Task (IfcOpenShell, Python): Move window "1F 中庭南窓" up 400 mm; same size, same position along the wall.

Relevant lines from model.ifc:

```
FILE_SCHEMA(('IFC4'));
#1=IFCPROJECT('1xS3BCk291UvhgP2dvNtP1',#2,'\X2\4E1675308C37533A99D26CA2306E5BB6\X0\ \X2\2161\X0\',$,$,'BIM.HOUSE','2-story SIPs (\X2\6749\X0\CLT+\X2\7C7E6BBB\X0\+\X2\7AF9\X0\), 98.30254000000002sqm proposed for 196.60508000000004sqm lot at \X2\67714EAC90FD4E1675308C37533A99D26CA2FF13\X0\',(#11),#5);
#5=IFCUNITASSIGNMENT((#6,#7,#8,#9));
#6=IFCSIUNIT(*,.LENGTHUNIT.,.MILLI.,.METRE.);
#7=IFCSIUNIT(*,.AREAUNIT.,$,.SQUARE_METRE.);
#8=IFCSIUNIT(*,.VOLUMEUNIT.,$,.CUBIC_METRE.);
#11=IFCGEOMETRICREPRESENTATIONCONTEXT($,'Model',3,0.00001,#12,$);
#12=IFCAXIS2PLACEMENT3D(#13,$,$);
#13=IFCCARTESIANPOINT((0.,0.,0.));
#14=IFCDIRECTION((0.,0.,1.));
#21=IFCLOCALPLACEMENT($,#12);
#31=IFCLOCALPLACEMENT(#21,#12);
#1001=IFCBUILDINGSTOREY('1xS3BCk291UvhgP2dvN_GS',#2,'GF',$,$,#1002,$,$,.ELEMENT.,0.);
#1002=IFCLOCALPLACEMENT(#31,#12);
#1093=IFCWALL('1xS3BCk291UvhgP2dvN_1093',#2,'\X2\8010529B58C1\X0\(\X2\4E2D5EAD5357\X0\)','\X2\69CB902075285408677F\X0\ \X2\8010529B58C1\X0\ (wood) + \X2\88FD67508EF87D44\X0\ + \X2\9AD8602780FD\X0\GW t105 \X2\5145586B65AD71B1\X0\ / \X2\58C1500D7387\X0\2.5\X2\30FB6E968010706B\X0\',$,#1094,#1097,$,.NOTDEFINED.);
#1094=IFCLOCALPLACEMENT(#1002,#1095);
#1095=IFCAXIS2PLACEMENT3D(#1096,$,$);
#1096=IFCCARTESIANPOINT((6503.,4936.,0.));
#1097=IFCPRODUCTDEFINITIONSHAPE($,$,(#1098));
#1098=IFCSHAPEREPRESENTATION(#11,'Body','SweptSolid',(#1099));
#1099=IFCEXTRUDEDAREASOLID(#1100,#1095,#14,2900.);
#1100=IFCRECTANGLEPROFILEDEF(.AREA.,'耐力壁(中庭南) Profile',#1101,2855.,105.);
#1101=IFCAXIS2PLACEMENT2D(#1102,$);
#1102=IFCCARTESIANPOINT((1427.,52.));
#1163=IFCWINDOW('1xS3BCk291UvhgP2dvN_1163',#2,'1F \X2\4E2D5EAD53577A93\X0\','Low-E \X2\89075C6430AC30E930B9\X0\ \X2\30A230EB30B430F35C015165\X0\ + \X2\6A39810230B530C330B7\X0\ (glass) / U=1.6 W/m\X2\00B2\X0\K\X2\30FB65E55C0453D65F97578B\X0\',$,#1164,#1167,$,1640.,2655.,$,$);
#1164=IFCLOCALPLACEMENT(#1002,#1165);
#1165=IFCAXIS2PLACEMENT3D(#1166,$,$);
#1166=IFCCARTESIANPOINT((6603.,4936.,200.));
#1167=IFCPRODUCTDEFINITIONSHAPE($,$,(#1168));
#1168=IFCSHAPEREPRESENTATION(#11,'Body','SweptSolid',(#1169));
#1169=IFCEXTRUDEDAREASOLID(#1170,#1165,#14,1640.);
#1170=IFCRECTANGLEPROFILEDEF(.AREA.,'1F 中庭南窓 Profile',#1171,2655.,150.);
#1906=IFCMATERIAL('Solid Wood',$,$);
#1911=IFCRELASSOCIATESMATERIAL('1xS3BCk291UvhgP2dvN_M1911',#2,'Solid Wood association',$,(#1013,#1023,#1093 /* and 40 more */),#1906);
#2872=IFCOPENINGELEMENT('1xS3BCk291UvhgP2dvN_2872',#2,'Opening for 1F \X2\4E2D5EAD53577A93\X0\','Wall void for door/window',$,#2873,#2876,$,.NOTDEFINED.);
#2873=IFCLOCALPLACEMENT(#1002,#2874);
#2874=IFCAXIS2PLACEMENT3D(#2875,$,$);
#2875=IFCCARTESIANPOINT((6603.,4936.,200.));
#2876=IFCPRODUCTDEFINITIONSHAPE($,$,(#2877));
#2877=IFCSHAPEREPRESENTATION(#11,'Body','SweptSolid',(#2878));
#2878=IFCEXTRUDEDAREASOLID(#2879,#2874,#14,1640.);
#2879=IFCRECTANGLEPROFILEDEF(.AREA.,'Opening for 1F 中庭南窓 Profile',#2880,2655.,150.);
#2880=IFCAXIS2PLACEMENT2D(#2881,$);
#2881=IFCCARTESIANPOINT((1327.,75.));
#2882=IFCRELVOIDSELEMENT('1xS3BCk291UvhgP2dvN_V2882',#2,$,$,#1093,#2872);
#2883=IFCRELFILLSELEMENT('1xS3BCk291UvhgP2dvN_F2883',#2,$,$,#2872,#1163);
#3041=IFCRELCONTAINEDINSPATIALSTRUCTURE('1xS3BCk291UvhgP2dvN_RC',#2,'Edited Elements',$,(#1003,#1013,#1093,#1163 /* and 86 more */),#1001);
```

```python
import numpy as np
import ifcopenshell
import ifcopenshell.api.geometry
import ifcopenshell.util.placement
import ifcopenshell.util.unit

model = ifcopenshell.open("model.ifc")
unit_scale = ifcopenshell.util.unit.calculate_unit_scale(model)

window = model.by_guid("1xS3BCk291UvhgP2dvN_1163")
opening = window.FillsVoids[0].RelatingOpeningElement
dz = 0.4 / unit_scale

shift = np.array([0.0, 0.0, dz])
# The window is not placed relative to its opening, so move both.
for product in (opening, window):
    matrix = ifcopenshell.util.placement.get_local_placement(product.ObjectPlacement)
    matrix[:3, 3] += shift
    ifcopenshell.api.geometry.edit_object_placement(model, product=product, matrix=matrix, is_si=False)

print(f"moved by {dz * unit_scale:+.3f} m")

model.write("model_edited.ifc")
```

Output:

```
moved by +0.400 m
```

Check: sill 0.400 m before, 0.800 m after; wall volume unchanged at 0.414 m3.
